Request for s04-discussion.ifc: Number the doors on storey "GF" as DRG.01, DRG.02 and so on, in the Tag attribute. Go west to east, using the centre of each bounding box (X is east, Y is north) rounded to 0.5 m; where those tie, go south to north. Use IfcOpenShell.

First a look at what the model holds.

```python
import ifcopenshell
import ifcopenshell.util.element
import ifcopenshell.util.placement

model = ifcopenshell.open("s04-discussion.ifc")
print(model.schema)
storey = next(s for s in model.by_type("IfcBuildingStorey") if s.Name == "GF")
doors = [e for e in ifcopenshell.util.element.get_decomposition(storey) if e.is_a("IfcDoor")]
for e in sorted(doors, key=lambda e: e.id()):
    origin = ifcopenshell.util.placement.get_local_placement(e.ObjectPlacement)[:3, 3]
    print(e.id(), e.Tag, e.Name, origin.round(2) + 0.0, sep=" | ")
```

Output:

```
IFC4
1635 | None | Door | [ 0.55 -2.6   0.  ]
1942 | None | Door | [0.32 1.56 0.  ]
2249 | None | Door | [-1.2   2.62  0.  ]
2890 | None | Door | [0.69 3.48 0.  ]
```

```python
import ifcopenshell
import ifcopenshell.geom
import ifcopenshell.util.element
import ifcopenshell.util.shape

model = ifcopenshell.open("s04-discussion.ifc")
settings = ifcopenshell.geom.settings()
settings.set("use-world-coords", True)


def centre(element):
    shape = ifcopenshell.geom.create_shape(settings, element)
    return ifcopenshell.util.shape.get_bbox_centroid(shape.geometry)


storey = next(s for s in model.by_type("IfcBuildingStorey") if s.Name == "GF")
doors = [e for e in ifcopenshell.util.element.get_decomposition(storey) if e.is_a("IfcDoor")]

# Insertion points can sit at a corner or the storey origin, so sort by the geometry (in metres).
centres = {e: centre(e) for e in doors}
doors.sort(key=lambda e: (round(centres[e][0] / 0.5), centres[e][1]))

for i, e in enumerate(doors, start=1):
    number = f"DRG.{i:02d}"
    e.Tag = number
    print(e.id(), number)

model.write("s04-discussion_updated.ifc")
```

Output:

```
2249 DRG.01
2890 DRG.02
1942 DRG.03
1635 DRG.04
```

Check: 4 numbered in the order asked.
